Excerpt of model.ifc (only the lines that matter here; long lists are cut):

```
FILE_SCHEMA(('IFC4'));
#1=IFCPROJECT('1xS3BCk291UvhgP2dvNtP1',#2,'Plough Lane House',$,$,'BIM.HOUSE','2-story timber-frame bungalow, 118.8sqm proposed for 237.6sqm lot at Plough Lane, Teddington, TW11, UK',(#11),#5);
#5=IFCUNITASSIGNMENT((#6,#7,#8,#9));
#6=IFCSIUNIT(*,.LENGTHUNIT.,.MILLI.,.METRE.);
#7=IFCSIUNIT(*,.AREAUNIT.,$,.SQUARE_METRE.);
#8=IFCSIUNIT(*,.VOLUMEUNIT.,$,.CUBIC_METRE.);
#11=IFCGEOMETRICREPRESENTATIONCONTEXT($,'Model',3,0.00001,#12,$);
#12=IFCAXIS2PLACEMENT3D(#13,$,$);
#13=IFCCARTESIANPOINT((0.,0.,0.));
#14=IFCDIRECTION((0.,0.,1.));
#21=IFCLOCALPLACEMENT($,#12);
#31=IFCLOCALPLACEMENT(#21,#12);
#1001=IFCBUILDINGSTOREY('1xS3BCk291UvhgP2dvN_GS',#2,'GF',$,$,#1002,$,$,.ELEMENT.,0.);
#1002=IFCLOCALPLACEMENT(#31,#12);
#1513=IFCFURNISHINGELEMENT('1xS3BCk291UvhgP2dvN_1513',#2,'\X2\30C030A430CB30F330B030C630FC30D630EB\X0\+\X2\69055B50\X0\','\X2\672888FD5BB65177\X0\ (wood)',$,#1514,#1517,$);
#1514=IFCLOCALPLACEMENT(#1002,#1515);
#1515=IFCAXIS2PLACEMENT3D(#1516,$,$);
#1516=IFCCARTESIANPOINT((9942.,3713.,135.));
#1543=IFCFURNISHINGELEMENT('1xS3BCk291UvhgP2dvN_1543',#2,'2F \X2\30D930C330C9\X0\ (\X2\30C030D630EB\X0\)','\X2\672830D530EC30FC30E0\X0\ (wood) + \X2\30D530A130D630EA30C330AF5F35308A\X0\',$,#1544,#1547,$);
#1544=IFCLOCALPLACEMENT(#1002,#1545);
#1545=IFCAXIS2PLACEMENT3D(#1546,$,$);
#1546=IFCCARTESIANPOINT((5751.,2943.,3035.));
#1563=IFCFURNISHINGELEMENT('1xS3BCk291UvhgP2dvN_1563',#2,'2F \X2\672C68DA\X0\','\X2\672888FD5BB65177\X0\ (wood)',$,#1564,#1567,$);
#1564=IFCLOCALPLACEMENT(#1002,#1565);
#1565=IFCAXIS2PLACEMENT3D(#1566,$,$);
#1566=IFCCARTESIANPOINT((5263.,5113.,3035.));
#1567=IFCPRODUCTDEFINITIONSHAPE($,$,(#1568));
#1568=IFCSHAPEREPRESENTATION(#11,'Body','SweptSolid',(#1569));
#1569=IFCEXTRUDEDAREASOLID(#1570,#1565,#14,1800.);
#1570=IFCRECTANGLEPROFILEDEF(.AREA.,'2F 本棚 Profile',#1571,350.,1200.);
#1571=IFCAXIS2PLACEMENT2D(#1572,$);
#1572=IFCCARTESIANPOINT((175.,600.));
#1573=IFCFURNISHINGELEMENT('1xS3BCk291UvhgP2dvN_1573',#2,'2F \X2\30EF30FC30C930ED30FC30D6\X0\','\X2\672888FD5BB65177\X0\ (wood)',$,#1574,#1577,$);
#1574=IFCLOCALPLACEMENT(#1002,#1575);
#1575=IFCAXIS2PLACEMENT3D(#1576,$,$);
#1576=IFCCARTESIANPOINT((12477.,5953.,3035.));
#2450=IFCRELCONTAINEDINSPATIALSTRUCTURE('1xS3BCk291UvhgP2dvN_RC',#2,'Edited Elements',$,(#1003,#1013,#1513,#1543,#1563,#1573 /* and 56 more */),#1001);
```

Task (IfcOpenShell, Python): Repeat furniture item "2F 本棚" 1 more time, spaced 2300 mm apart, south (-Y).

```python
import numpy as np
import ifcopenshell
import ifcopenshell.api.geometry
import ifcopenshell.api.root
import ifcopenshell.util.element
import ifcopenshell.util.placement
import ifcopenshell.util.unit

model = ifcopenshell.open("model.ifc")
unit_scale = ifcopenshell.util.unit.calculate_unit_scale(model)


def reuse_history(source, copy):
    """copy_class also copies each property set's owner history, people and application; keep the originals."""
    for rel in copy.IsDefinedBy:
        if rel.is_a("IfcRelDefinesByProperties") and (history := rel.RelatingPropertyDefinition.OwnerHistory):
            rel.RelatingPropertyDefinition.OwnerHistory = source.OwnerHistory
            ifcopenshell.util.element.remove_deep2(model, history)


source = model.by_id(1563)
base = ifcopenshell.util.placement.get_local_placement(source.ObjectPlacement)
step = np.array([0.0, -1.0, 0.0]) * 2.3 / unit_scale

for i in range(1, 2):
    copy = ifcopenshell.api.root.copy_class(model, product=source)
    copy.Representation = ifcopenshell.util.element.copy_deep(
        model, source.Representation, exclude=["IfcGeometricRepresentationContext", "IfcRepresentationMap"]
    )
    reuse_history(source, copy)
    matrix = base.copy()
    matrix[:3, 3] += i * step
    print("added at", matrix[:3, 3].round(3) + 0.0)
    ifcopenshell.api.geometry.edit_object_placement(model, product=copy, matrix=matrix, is_si=False)

model.write("model_updated.ifc")
```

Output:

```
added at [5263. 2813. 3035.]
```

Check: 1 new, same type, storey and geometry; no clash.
